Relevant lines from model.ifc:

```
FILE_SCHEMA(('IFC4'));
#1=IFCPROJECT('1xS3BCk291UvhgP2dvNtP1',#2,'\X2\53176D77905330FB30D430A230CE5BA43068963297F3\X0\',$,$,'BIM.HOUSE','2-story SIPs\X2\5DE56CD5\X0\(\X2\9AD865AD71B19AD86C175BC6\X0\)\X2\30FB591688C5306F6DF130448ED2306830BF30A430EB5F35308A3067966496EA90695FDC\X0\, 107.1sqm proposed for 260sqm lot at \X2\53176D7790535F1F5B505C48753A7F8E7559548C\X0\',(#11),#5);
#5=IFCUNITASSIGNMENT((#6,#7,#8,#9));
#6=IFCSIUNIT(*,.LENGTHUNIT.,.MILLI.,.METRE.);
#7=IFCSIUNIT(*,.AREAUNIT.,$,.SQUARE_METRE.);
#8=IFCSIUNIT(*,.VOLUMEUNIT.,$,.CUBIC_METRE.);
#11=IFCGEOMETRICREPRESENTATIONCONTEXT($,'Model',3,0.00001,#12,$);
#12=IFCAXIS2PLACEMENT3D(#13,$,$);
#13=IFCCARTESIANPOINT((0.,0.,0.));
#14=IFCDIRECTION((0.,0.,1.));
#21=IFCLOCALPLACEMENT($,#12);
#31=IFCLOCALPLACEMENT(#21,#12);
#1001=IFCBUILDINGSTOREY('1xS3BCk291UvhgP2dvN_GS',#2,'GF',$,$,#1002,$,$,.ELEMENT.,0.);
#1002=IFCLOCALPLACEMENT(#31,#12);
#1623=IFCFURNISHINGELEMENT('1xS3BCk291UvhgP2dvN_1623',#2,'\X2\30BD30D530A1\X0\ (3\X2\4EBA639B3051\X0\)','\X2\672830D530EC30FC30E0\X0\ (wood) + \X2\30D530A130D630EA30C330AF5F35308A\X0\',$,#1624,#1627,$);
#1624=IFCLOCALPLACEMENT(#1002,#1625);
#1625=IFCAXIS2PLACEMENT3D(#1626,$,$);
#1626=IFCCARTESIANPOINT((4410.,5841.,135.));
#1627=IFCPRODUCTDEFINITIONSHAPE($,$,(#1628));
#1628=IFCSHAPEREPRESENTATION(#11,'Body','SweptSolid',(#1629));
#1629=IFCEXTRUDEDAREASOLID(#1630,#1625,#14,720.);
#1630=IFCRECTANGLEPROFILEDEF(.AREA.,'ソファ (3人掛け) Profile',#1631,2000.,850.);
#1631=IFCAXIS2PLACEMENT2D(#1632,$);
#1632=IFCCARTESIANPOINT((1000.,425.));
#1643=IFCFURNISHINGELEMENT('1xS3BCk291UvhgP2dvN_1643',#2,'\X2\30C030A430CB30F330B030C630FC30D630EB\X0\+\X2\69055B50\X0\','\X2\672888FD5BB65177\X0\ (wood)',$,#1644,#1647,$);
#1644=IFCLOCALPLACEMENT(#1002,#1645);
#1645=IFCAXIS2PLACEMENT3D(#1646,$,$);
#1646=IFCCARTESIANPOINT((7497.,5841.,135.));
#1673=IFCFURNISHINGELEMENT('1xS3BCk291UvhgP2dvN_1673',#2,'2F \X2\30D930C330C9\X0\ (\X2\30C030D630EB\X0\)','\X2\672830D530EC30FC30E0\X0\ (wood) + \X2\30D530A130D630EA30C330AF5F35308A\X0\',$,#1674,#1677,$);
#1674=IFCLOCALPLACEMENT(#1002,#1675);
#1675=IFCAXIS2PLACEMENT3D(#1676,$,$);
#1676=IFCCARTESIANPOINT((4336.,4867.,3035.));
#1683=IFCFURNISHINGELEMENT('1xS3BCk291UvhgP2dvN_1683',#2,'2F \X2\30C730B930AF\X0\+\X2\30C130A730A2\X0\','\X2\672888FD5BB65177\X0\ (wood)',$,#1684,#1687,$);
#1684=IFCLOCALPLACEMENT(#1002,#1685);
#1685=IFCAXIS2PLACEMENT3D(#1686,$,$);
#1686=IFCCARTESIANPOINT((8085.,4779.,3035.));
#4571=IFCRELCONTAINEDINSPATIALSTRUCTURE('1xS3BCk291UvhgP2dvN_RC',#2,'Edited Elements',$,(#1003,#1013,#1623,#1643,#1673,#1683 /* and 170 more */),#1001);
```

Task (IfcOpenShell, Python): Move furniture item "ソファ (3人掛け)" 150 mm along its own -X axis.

```python
import ifcopenshell
import ifcopenshell.api.geometry
import ifcopenshell.util.placement

model = ifcopenshell.open("model.ifc")

item = model.by_id(1623)
matrix = ifcopenshell.util.placement.get_local_placement(item.ObjectPlacement)
matrix[:3, 3] -= matrix[:3, 0] * 150.0
ifcopenshell.api.geometry.edit_object_placement(model, product=item, matrix=matrix, is_si=False)

print(ifcopenshell.util.placement.get_local_placement(item.ObjectPlacement).round(3) + 0.0)

model.write("model_updated.ifc")
```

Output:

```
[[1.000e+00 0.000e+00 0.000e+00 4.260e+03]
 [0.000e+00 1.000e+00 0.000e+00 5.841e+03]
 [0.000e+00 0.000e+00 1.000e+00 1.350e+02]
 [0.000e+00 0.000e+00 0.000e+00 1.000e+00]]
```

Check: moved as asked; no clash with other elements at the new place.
